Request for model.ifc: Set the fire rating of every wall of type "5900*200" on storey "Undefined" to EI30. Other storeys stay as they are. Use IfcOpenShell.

First a look at what the model holds.

```python
import ifcopenshell
import ifcopenshell.util.element

model = ifcopenshell.open("model.ifc")
print(model.schema)
storey = next(s for s in model.by_type("IfcBuildingStorey") if s.Name == "Undefined")
walls = [e for e in ifcopenshell.util.element.get_decomposition(storey) if e.is_a("IfcWall")]
seen = {}
for e in walls:
    element_type = ifcopenshell.util.element.get_type(e)
    key = (element_type.Name if element_type != e and element_type else None, ifcopenshell.util.element.get_pset(e, "Pset_WallCommon", "FireRating"))
    seen[key] = seen.get(key, 0) + 1
for (name, value), count in sorted(seen.items(), key=str):
    print(count, "x", name, "|", value)
```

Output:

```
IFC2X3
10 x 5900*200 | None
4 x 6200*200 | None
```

```python
import ifcopenshell
import ifcopenshell.api.pset
import ifcopenshell.util.element

model = ifcopenshell.open("model.ifc")

storey = next(s for s in model.by_type("IfcBuildingStorey") if s.Name == "Undefined")
walls = [e for e in ifcopenshell.util.element.get_decomposition(storey) if e.is_a("IfcWall")]

count = 0
for e in walls:
    element_type = ifcopenshell.util.element.get_type(e)
    if element_type in (None, e) or element_type.Name != "5900*200":
        continue
    # add_pset returns the element's existing set when there is one.
    pset = ifcopenshell.api.pset.add_pset(model, product=e, name="Pset_WallCommon")
    ifcopenshell.api.pset.edit_pset(model, pset=pset, properties={"FireRating": "EI30"})
    count += 1

print(count, "walls updated")

model.write("model_edited.ifc")
```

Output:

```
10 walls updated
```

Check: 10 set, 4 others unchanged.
